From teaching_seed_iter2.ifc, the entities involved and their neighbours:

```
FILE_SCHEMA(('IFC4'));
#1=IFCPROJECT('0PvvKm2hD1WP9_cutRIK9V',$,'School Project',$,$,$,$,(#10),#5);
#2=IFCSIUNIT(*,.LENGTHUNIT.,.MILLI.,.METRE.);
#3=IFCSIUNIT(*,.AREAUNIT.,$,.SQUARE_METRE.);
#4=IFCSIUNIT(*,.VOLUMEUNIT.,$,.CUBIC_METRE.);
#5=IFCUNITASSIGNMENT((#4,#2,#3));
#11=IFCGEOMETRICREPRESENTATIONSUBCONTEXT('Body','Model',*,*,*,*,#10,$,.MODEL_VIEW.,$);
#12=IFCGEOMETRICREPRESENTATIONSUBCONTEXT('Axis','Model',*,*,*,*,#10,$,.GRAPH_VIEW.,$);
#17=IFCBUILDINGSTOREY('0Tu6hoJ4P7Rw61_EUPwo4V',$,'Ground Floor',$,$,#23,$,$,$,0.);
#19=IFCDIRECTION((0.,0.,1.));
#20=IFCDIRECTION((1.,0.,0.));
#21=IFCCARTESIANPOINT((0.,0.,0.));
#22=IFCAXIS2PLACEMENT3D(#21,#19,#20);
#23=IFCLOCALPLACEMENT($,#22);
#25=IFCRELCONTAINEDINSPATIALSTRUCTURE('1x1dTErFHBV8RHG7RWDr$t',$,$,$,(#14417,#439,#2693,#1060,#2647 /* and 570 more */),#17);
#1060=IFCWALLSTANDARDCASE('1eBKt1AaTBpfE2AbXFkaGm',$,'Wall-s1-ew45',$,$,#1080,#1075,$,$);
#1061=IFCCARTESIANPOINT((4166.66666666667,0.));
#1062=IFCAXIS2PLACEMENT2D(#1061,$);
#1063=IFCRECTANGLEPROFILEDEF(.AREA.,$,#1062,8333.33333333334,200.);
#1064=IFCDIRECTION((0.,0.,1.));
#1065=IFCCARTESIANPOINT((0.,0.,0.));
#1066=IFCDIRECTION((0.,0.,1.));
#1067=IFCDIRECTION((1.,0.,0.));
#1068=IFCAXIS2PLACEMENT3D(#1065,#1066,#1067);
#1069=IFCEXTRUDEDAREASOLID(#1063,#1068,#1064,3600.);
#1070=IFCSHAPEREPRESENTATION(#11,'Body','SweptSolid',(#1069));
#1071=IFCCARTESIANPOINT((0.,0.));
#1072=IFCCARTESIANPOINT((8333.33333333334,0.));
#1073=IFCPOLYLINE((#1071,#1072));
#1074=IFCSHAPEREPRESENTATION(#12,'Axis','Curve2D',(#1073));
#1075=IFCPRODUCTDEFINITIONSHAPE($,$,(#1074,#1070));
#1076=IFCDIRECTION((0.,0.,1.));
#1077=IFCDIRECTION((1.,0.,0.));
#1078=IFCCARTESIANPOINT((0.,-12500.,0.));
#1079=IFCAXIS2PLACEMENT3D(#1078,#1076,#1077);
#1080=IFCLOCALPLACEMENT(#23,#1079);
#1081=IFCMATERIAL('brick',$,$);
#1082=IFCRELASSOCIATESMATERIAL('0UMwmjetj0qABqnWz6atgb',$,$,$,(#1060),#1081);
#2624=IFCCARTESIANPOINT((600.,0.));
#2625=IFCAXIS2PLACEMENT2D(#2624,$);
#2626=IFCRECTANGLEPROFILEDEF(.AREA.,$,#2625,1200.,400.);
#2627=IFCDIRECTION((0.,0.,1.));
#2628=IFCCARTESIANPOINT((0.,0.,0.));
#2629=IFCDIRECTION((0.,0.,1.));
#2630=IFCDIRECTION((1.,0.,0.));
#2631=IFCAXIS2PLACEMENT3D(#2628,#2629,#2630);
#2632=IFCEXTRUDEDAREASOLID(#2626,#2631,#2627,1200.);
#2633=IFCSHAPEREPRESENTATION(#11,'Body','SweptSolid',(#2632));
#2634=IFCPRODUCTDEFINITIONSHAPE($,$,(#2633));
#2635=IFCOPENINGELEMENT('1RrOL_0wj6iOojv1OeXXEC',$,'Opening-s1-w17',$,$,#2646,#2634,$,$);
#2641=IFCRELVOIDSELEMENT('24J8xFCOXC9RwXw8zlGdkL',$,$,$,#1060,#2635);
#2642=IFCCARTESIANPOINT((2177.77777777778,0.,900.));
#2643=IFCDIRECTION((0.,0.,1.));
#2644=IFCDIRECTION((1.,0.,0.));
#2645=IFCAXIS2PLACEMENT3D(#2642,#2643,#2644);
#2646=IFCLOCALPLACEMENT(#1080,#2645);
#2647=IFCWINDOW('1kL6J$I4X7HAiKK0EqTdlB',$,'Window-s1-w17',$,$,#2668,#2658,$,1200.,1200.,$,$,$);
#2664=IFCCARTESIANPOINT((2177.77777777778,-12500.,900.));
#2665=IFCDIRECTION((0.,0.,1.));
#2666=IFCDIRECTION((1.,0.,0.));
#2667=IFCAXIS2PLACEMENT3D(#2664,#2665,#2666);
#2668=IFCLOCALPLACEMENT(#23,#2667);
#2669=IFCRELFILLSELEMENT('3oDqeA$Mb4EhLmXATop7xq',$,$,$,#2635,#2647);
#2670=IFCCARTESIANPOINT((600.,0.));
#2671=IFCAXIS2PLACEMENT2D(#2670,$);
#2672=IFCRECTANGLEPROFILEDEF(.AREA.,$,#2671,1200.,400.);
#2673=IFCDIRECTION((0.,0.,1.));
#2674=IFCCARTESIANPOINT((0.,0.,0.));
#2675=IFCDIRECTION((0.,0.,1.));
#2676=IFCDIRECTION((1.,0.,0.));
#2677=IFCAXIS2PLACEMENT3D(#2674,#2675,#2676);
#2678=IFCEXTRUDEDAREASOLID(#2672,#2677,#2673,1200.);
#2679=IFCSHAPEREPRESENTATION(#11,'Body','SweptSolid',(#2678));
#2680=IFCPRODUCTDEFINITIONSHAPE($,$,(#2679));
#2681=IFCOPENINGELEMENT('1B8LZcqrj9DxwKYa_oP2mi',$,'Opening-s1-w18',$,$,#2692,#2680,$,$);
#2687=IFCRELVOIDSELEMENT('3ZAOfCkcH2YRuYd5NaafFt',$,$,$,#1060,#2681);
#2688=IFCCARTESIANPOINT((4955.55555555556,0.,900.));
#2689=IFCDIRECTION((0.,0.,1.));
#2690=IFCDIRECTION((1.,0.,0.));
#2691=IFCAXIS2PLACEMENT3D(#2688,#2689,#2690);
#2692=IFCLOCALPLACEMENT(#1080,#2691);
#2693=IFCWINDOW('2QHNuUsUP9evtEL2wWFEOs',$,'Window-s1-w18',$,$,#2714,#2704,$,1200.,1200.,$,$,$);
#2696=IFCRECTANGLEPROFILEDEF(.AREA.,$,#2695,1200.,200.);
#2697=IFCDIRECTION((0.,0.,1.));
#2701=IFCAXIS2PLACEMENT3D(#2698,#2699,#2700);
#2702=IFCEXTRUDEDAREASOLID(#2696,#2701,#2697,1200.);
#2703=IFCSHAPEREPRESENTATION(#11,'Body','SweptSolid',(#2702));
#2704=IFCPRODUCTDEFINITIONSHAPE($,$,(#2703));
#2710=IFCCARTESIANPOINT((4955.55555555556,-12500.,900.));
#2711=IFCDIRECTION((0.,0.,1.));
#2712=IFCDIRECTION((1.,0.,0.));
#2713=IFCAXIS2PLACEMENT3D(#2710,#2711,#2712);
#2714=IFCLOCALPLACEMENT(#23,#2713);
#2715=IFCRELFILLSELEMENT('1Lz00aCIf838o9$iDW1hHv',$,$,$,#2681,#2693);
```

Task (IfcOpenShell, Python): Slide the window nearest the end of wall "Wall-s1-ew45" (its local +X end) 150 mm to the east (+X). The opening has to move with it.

```python
import ifcopenshell
import ifcopenshell.api.geometry
import ifcopenshell.util.placement
import ifcopenshell.util.unit

model = ifcopenshell.open("teaching_seed_iter2.ifc")
unit_scale = ifcopenshell.util.unit.calculate_unit_scale(model)

window = model.by_guid("2QHNuUsUP9evtEL2wWFEOs")
opening = window.FillsVoids[0].RelatingOpeningElement
wall = opening.VoidsElements[0].RelatingBuildingElement

wall_matrix = ifcopenshell.util.placement.get_local_placement(wall.ObjectPlacement)
shift = wall_matrix[:3, 0] * 0.15 / unit_scale
before = ifcopenshell.util.placement.get_local_placement(window.ObjectPlacement)[:3, 3].copy()

# The window is not placed relative to its opening, so move both.
for product in (opening, window):
    matrix = ifcopenshell.util.placement.get_local_placement(product.ObjectPlacement)
    matrix[:3, 3] += shift
    ifcopenshell.api.geometry.edit_object_placement(model, product=product, matrix=matrix, is_si=False)

after = ifcopenshell.util.placement.get_local_placement(window.ObjectPlacement)[:3, 3]
print("window moved by", (after - before).round(3) + 0.0)

model.write("teaching_seed_iter2_updated.ifc")
```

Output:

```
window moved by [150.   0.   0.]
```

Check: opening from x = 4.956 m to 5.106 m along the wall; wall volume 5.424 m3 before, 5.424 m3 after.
